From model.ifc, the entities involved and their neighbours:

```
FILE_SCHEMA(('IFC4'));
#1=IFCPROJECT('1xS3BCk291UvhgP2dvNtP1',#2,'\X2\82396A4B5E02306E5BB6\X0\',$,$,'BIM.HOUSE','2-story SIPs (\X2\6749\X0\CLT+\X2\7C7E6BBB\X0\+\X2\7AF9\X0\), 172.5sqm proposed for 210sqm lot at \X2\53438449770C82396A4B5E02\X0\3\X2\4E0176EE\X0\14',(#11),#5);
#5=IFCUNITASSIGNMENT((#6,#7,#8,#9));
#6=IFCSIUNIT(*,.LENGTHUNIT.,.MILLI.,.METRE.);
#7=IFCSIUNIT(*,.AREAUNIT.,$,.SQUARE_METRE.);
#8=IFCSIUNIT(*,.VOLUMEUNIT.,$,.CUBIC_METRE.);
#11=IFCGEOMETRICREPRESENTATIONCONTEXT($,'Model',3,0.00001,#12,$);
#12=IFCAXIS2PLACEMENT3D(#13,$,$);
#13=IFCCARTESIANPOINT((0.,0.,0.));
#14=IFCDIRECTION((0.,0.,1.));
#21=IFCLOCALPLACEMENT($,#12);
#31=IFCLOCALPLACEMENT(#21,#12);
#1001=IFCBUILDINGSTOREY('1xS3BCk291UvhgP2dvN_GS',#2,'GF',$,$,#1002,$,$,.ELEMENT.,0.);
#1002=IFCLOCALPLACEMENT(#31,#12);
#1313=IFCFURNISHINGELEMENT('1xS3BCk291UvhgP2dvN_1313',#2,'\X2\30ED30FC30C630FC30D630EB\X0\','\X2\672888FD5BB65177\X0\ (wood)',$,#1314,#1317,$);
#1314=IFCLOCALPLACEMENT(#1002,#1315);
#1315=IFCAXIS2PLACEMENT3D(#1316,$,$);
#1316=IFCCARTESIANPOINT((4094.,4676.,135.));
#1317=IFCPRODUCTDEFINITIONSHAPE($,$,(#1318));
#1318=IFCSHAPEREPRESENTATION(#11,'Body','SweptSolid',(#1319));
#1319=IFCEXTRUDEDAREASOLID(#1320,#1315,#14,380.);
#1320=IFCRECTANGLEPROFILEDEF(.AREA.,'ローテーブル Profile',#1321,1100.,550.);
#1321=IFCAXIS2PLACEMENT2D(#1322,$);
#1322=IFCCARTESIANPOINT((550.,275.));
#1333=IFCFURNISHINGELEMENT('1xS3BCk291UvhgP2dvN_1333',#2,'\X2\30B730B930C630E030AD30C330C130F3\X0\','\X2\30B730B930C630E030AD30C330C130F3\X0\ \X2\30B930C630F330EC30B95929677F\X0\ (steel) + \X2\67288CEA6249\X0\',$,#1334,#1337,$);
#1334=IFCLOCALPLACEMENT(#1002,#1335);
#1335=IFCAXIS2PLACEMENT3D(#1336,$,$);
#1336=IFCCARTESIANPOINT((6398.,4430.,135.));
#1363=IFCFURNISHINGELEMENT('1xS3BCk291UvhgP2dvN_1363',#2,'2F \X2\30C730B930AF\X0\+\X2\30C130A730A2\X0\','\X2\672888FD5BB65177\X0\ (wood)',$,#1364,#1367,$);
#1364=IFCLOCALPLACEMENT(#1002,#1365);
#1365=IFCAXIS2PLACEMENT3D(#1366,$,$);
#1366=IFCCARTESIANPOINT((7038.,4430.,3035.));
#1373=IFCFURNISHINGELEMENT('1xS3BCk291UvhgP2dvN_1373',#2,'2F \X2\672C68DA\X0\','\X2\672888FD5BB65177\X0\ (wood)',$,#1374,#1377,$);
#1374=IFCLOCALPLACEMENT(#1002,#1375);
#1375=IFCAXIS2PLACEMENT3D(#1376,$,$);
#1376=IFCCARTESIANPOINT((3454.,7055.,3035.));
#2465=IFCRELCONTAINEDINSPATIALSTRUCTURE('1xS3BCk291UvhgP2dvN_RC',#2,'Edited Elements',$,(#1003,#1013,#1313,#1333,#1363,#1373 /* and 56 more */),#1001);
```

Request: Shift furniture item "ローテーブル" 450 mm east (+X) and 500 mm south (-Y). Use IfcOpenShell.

```python
import ifcopenshell
import ifcopenshell.api.geometry
import ifcopenshell.util.placement

model = ifcopenshell.open("model.ifc")

item = model.by_guid("1xS3BCk291UvhgP2dvN_1313")
matrix = ifcopenshell.util.placement.get_local_placement(item.ObjectPlacement)
matrix[0, 3] += 450.0
matrix[1, 3] -= 500.0
ifcopenshell.api.geometry.edit_object_placement(model, product=item, matrix=matrix, is_si=False)

print(ifcopenshell.util.placement.get_local_placement(item.ObjectPlacement).round(3) + 0.0)

model.write("model_updated.ifc")
```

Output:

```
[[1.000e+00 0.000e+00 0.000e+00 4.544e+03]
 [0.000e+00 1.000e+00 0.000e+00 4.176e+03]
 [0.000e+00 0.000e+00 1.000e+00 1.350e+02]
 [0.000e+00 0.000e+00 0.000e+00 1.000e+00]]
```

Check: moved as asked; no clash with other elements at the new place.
